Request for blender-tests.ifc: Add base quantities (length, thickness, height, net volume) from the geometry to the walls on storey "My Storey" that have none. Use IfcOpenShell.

First a look at what the model holds.

```python
import ifcopenshell
import ifcopenshell.util.element
import ifcopenshell.util.unit

model = ifcopenshell.open("blender-tests.ifc")
print(model.schema)
for unit_type in ("LENGTHUNIT", "AREAUNIT", "VOLUMEUNIT"):
    print(unit_type, ifcopenshell.util.unit.calculate_unit_scale(model, unit_type))
storey = next(s for s in model.by_type("IfcBuildingStorey") if s.Name == "My Storey")
walls = [e for e in ifcopenshell.util.element.get_decomposition(storey) if e.is_a("IfcWall")]
for e in sorted(walls, key=lambda e: e.id()):
    print(e.id(), e.is_a(), e.Name, list(ifcopenshell.util.element.get_psets(e, qtos_only=True)), sep=" | ")
```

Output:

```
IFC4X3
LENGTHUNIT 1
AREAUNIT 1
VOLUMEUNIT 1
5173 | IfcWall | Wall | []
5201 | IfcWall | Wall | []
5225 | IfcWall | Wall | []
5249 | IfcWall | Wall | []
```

```python
import ifcopenshell
import ifcopenshell.api.pset
import ifcopenshell.geom
import ifcopenshell.util.element
import ifcopenshell.util.shape
import ifcopenshell.util.unit

model = ifcopenshell.open("blender-tests.ifc")
unit_scale = ifcopenshell.util.unit.calculate_unit_scale(model)
volume_scale = ifcopenshell.util.unit.calculate_unit_scale(model, "VOLUMEUNIT")
settings = ifcopenshell.geom.settings()

storey = next(s for s in model.by_type("IfcBuildingStorey") if s.Name == "My Storey")
walls = [e for e in ifcopenshell.util.element.get_decomposition(storey) if e.is_a("IfcWall")]

for e in sorted(walls, key=lambda e: e.id()):
    if ifcopenshell.util.element.get_psets(e, qtos_only=True, should_inherit=False):
        continue
    # Geometry comes back in metres, in the element's own axes.
    shape = ifcopenshell.geom.create_shape(settings, e)
    values = {
        "Length": ifcopenshell.util.shape.get_x(shape.geometry) / unit_scale,
        "Width": ifcopenshell.util.shape.get_y(shape.geometry) / unit_scale,
        "Height": ifcopenshell.util.shape.get_z(shape.geometry) / unit_scale,
        "NetVolume": ifcopenshell.util.shape.get_volume(shape.geometry) / volume_scale,
    }
    qto = ifcopenshell.api.pset.add_qto(model, product=e, name="Qto_WallBaseQuantities")
    ifcopenshell.api.pset.edit_qto(model, qto=qto, properties=values)
    print(e.id(), {k: round(v, 3) for k, v in values.items()})

model.write("blender-tests-out.ifc")
```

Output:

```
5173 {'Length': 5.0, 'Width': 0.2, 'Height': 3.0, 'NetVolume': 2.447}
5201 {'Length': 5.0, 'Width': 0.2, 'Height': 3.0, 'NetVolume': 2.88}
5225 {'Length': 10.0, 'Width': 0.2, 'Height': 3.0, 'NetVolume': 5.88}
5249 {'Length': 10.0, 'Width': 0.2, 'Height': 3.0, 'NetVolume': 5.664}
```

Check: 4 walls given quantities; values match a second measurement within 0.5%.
